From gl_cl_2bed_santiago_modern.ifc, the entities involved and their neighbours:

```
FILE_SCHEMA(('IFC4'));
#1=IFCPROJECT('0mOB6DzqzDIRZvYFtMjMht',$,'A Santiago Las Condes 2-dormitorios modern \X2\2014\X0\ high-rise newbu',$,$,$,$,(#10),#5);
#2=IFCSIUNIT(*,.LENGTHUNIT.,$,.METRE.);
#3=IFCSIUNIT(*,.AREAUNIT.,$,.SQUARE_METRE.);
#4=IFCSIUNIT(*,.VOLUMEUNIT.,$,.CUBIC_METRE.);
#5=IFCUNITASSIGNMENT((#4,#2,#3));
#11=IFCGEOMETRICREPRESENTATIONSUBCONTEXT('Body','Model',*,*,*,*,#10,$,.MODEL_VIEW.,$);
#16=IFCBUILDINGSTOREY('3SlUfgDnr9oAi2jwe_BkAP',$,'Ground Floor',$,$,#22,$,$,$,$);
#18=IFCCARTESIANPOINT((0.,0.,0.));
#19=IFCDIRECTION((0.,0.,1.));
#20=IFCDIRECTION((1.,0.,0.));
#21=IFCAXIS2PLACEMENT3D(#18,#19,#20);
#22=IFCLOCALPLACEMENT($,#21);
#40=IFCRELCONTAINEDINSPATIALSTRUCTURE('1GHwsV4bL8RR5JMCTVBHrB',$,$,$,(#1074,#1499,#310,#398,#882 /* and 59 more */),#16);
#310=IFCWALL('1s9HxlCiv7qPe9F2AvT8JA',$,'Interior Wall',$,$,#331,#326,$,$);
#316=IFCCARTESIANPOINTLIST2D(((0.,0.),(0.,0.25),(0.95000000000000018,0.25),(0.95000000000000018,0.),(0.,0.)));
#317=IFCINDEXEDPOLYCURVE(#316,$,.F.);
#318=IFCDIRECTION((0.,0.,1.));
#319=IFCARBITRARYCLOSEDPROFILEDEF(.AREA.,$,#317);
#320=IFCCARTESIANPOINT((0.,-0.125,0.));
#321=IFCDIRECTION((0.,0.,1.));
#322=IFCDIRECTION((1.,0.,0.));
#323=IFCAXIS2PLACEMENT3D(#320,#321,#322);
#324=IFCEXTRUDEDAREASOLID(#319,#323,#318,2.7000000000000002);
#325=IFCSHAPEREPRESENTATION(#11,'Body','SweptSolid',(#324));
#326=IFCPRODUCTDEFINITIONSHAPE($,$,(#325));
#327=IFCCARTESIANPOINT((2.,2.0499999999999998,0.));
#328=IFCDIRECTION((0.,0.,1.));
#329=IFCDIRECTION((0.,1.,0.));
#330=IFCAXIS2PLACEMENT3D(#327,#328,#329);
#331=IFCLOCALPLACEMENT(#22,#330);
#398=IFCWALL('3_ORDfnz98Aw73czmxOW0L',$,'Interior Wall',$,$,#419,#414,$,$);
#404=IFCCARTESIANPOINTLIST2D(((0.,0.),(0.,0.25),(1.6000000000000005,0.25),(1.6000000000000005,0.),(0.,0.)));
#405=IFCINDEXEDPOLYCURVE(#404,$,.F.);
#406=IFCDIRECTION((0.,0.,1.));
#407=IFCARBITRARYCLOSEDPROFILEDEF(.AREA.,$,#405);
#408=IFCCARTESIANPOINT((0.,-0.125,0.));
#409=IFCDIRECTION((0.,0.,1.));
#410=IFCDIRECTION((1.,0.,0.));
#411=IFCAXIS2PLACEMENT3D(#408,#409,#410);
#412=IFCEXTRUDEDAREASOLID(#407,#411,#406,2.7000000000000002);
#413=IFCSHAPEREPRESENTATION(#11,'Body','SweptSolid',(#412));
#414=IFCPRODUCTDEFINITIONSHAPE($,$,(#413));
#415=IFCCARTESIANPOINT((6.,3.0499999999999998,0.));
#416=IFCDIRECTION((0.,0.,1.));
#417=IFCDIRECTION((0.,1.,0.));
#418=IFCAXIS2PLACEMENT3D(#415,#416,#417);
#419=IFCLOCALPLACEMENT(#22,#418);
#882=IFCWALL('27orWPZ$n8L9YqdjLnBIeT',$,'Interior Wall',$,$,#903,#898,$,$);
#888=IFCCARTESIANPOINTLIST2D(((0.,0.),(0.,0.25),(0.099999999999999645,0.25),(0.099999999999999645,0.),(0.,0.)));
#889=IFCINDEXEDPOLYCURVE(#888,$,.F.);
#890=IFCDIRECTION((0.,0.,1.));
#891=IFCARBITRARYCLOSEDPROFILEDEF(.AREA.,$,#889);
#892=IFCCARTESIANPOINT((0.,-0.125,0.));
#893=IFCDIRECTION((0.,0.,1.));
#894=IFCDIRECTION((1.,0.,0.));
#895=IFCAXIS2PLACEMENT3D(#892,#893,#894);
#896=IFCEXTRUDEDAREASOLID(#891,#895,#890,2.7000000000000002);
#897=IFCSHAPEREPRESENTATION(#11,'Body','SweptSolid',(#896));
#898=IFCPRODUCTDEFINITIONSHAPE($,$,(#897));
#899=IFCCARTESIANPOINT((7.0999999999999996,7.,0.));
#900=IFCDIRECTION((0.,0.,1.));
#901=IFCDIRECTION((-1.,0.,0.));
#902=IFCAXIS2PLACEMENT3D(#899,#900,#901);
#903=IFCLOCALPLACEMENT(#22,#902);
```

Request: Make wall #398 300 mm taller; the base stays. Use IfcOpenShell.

```python
import ifcopenshell
import ifcopenshell.geom
import ifcopenshell.util.representation
import ifcopenshell.util.shape
import ifcopenshell.util.unit

model = ifcopenshell.open("gl_cl_2bed_santiago_modern.ifc")
unit_scale = ifcopenshell.util.unit.calculate_unit_scale(model)
settings = ifcopenshell.geom.settings()


def volume(element):
    """Net volume in cubic metres, openings subtracted."""
    shape = ifcopenshell.geom.create_shape(settings, element)
    return ifcopenshell.util.shape.get_volume(shape.geometry)


wall = model.by_guid("3_ORDfnz98Aw73czmxOW0L")
before = volume(wall)

body = ifcopenshell.util.representation.get_representation(wall, "Model", "Body")
solid = body.Items[0]
old_height = solid.Depth
solid.Depth += 0.3 / unit_scale
after = volume(wall)

print(f"height {old_height:g} -> {solid.Depth:g}, volume {before:.3f} -> {after:.3f} m3")

model.write("gl_cl_2bed_santiago_modern_rev.ifc")
```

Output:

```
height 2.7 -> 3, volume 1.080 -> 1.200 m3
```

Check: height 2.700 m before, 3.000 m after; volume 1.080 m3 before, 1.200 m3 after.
